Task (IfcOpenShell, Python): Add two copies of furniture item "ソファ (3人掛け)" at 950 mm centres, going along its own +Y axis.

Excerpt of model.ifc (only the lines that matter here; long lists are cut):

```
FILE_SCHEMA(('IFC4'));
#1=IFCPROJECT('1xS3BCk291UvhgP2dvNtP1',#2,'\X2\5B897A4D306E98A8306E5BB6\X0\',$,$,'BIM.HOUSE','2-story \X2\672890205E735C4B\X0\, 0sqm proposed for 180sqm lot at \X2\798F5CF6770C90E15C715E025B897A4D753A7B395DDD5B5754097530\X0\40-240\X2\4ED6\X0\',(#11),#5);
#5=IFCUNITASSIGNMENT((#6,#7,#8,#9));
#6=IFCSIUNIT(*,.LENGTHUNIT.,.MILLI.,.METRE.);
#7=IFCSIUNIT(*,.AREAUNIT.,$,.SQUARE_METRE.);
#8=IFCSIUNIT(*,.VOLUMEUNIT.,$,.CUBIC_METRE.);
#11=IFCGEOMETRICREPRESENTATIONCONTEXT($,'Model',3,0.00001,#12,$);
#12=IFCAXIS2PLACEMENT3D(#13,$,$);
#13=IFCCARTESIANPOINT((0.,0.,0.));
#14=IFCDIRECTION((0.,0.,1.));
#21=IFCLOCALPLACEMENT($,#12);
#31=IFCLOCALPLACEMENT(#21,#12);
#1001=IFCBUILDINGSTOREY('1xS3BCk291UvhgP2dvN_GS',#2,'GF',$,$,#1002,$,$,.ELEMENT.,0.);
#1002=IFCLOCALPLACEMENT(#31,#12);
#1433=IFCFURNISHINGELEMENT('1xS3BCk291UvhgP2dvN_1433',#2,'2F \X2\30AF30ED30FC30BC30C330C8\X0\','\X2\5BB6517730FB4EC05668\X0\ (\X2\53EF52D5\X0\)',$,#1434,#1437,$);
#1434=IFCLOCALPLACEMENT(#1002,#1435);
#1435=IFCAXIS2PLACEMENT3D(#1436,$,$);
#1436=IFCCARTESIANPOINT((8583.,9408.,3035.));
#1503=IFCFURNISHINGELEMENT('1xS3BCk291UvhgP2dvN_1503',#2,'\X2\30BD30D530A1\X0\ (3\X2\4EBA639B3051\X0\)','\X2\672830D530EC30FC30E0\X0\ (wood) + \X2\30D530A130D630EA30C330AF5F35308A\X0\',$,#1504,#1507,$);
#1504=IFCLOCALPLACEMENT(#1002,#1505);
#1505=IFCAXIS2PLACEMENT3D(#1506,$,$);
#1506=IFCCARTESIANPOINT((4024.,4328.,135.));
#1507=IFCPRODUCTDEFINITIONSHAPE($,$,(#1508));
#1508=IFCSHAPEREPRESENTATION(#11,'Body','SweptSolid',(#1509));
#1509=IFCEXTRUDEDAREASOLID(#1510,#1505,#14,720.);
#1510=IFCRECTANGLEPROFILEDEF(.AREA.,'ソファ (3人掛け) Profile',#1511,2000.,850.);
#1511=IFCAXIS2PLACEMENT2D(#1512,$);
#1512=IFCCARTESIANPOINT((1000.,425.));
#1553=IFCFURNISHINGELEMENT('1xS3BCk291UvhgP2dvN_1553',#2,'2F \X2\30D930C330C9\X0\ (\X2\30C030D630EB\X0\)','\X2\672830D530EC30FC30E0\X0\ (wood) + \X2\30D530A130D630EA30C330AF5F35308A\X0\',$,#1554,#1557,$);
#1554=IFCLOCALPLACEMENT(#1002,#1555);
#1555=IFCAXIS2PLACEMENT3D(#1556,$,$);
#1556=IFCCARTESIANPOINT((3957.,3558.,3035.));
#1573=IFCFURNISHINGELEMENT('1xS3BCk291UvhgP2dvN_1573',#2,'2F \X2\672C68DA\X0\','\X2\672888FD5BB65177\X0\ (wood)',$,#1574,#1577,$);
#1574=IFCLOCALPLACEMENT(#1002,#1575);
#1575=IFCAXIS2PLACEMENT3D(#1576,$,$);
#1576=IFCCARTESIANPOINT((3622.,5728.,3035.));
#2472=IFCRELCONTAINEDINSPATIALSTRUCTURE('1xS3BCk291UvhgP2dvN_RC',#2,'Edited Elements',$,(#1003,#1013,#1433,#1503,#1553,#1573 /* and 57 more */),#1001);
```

```python
import ifcopenshell
import ifcopenshell.api.geometry
import ifcopenshell.api.root
import ifcopenshell.util.element
import ifcopenshell.util.placement
import ifcopenshell.util.unit

model = ifcopenshell.open("model.ifc")
unit_scale = ifcopenshell.util.unit.calculate_unit_scale(model)


def reuse_history(source, copy):
    """copy_class also copies each property set's owner history, people and application; keep the originals."""
    for rel in copy.IsDefinedBy:
        if rel.is_a("IfcRelDefinesByProperties") and (history := rel.RelatingPropertyDefinition.OwnerHistory):
            rel.RelatingPropertyDefinition.OwnerHistory = source.OwnerHistory
            ifcopenshell.util.element.remove_deep2(model, history)


source = model.by_guid("1xS3BCk291UvhgP2dvN_1503")
base = ifcopenshell.util.placement.get_local_placement(source.ObjectPlacement)
step = base[:3, 1] * 0.95 / unit_scale

for i in range(1, 3):
    copy = ifcopenshell.api.root.copy_class(model, product=source)
    copy.Representation = ifcopenshell.util.element.copy_deep(
        model, source.Representation, exclude=["IfcGeometricRepresentationContext", "IfcRepresentationMap"]
    )
    reuse_history(source, copy)
    matrix = base.copy()
    matrix[:3, 3] += i * step
    print("added at", matrix[:3, 3].round(3) + 0.0)
    ifcopenshell.api.geometry.edit_object_placement(model, product=copy, matrix=matrix, is_si=False)

model.write("model_edited.ifc")
```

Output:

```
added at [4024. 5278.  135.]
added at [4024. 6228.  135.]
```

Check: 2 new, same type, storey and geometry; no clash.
